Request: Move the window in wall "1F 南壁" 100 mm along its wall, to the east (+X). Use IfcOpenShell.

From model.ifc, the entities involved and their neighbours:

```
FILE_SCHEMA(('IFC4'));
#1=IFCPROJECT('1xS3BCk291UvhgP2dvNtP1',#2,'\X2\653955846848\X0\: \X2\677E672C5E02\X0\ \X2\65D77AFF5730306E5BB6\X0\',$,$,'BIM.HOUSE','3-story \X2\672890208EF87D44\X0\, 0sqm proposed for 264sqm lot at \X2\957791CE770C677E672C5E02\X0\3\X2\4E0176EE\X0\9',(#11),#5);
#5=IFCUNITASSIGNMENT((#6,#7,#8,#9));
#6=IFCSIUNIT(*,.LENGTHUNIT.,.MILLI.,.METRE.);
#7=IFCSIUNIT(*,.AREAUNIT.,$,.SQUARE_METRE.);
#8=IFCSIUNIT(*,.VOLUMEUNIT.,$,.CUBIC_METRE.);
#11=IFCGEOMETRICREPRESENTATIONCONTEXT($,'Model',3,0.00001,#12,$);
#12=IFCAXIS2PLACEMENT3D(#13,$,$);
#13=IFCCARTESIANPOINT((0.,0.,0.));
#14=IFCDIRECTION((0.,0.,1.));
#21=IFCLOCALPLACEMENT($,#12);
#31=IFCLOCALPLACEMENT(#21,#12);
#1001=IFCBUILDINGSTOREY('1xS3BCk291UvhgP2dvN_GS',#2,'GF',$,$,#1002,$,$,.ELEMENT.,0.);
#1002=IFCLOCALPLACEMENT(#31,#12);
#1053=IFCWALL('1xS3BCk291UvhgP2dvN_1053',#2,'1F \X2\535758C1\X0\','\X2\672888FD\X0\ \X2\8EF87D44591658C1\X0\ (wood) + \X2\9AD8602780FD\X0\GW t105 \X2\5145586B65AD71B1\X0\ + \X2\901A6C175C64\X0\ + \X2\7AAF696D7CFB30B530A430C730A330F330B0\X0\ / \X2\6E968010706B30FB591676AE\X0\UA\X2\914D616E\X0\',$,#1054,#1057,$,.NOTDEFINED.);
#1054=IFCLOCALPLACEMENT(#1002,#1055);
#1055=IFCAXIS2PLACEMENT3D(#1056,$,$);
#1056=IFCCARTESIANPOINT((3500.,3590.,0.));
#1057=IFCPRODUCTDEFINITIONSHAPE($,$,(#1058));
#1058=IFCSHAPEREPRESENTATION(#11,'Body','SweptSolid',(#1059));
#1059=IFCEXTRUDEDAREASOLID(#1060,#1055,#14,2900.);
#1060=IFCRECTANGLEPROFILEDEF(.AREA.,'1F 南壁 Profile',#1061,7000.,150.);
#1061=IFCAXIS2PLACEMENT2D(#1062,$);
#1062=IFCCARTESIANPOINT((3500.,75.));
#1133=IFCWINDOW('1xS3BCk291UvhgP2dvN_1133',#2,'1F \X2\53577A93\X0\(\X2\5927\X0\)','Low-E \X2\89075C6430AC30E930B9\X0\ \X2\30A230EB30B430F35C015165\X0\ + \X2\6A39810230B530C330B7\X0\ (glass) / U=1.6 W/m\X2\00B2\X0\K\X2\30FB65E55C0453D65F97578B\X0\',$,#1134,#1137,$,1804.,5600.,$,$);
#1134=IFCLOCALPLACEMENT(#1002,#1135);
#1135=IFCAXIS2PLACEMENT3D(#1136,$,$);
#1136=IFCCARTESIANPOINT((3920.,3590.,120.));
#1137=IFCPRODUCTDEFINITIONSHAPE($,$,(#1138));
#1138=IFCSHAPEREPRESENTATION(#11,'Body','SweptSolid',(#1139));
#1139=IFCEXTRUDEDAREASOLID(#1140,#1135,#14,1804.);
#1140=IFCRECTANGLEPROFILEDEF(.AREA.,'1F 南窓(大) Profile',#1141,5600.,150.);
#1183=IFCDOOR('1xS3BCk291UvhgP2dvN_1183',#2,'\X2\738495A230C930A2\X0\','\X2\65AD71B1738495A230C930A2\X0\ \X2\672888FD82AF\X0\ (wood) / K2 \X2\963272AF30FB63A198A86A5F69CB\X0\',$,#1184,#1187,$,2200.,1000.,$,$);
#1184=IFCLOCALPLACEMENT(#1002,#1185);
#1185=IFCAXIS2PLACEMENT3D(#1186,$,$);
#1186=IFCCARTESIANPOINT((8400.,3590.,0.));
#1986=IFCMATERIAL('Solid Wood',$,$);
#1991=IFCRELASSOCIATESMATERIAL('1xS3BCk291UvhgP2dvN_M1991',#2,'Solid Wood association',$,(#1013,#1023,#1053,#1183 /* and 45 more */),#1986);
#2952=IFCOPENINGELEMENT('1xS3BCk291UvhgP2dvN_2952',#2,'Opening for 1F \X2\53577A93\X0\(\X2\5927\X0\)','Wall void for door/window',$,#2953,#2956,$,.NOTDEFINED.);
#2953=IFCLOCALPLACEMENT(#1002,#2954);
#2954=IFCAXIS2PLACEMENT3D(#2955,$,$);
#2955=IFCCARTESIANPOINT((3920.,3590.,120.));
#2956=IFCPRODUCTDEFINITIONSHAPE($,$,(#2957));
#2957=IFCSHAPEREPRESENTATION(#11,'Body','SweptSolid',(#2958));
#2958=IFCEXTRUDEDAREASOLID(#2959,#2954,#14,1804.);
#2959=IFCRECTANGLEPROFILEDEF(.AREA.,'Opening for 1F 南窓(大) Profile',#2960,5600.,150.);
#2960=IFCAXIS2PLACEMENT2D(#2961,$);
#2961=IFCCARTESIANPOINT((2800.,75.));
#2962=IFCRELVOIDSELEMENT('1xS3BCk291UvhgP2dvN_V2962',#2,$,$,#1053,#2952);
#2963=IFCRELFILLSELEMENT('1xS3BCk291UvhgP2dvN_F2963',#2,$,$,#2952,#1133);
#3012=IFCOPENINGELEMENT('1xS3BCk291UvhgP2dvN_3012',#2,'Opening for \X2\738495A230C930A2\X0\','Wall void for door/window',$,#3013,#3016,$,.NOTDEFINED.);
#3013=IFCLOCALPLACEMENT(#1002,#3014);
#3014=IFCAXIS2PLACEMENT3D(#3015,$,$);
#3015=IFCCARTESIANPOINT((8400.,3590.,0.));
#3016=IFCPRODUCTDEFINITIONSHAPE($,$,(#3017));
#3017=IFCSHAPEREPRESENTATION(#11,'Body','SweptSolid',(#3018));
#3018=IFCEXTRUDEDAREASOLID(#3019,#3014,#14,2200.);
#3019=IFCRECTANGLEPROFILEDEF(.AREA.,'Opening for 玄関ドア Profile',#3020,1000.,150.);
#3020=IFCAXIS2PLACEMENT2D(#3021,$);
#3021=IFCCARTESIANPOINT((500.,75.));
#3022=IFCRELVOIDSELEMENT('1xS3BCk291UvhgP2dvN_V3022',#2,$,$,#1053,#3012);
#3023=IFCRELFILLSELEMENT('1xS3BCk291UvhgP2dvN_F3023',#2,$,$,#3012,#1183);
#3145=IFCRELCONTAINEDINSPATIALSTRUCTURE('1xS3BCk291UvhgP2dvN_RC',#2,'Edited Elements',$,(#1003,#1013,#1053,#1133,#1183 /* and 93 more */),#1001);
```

```python
import ifcopenshell
import ifcopenshell.api.geometry
import ifcopenshell.util.placement

model = ifcopenshell.open("model.ifc")

window = model.by_guid("1xS3BCk291UvhgP2dvN_1133")
opening = window.FillsVoids[0].RelatingOpeningElement
wall = opening.VoidsElements[0].RelatingBuildingElement

wall_matrix = ifcopenshell.util.placement.get_local_placement(wall.ObjectPlacement)
shift = wall_matrix[:3, 0] * 100.0
before = ifcopenshell.util.placement.get_local_placement(window.ObjectPlacement)[:3, 3].copy()

# The window is not placed relative to its opening, so move both.
for product in (opening, window):
    matrix = ifcopenshell.util.placement.get_local_placement(product.ObjectPlacement)
    matrix[:3, 3] += shift
    ifcopenshell.api.geometry.edit_object_placement(model, product=product, matrix=matrix, is_si=False)

after = ifcopenshell.util.placement.get_local_placement(window.ObjectPlacement)[:3, 3]
print("window moved by", (after - before).round(3) + 0.0)

model.write("model_updated.ifc")
```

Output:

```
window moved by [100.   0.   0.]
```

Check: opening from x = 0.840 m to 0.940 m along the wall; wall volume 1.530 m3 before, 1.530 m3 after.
